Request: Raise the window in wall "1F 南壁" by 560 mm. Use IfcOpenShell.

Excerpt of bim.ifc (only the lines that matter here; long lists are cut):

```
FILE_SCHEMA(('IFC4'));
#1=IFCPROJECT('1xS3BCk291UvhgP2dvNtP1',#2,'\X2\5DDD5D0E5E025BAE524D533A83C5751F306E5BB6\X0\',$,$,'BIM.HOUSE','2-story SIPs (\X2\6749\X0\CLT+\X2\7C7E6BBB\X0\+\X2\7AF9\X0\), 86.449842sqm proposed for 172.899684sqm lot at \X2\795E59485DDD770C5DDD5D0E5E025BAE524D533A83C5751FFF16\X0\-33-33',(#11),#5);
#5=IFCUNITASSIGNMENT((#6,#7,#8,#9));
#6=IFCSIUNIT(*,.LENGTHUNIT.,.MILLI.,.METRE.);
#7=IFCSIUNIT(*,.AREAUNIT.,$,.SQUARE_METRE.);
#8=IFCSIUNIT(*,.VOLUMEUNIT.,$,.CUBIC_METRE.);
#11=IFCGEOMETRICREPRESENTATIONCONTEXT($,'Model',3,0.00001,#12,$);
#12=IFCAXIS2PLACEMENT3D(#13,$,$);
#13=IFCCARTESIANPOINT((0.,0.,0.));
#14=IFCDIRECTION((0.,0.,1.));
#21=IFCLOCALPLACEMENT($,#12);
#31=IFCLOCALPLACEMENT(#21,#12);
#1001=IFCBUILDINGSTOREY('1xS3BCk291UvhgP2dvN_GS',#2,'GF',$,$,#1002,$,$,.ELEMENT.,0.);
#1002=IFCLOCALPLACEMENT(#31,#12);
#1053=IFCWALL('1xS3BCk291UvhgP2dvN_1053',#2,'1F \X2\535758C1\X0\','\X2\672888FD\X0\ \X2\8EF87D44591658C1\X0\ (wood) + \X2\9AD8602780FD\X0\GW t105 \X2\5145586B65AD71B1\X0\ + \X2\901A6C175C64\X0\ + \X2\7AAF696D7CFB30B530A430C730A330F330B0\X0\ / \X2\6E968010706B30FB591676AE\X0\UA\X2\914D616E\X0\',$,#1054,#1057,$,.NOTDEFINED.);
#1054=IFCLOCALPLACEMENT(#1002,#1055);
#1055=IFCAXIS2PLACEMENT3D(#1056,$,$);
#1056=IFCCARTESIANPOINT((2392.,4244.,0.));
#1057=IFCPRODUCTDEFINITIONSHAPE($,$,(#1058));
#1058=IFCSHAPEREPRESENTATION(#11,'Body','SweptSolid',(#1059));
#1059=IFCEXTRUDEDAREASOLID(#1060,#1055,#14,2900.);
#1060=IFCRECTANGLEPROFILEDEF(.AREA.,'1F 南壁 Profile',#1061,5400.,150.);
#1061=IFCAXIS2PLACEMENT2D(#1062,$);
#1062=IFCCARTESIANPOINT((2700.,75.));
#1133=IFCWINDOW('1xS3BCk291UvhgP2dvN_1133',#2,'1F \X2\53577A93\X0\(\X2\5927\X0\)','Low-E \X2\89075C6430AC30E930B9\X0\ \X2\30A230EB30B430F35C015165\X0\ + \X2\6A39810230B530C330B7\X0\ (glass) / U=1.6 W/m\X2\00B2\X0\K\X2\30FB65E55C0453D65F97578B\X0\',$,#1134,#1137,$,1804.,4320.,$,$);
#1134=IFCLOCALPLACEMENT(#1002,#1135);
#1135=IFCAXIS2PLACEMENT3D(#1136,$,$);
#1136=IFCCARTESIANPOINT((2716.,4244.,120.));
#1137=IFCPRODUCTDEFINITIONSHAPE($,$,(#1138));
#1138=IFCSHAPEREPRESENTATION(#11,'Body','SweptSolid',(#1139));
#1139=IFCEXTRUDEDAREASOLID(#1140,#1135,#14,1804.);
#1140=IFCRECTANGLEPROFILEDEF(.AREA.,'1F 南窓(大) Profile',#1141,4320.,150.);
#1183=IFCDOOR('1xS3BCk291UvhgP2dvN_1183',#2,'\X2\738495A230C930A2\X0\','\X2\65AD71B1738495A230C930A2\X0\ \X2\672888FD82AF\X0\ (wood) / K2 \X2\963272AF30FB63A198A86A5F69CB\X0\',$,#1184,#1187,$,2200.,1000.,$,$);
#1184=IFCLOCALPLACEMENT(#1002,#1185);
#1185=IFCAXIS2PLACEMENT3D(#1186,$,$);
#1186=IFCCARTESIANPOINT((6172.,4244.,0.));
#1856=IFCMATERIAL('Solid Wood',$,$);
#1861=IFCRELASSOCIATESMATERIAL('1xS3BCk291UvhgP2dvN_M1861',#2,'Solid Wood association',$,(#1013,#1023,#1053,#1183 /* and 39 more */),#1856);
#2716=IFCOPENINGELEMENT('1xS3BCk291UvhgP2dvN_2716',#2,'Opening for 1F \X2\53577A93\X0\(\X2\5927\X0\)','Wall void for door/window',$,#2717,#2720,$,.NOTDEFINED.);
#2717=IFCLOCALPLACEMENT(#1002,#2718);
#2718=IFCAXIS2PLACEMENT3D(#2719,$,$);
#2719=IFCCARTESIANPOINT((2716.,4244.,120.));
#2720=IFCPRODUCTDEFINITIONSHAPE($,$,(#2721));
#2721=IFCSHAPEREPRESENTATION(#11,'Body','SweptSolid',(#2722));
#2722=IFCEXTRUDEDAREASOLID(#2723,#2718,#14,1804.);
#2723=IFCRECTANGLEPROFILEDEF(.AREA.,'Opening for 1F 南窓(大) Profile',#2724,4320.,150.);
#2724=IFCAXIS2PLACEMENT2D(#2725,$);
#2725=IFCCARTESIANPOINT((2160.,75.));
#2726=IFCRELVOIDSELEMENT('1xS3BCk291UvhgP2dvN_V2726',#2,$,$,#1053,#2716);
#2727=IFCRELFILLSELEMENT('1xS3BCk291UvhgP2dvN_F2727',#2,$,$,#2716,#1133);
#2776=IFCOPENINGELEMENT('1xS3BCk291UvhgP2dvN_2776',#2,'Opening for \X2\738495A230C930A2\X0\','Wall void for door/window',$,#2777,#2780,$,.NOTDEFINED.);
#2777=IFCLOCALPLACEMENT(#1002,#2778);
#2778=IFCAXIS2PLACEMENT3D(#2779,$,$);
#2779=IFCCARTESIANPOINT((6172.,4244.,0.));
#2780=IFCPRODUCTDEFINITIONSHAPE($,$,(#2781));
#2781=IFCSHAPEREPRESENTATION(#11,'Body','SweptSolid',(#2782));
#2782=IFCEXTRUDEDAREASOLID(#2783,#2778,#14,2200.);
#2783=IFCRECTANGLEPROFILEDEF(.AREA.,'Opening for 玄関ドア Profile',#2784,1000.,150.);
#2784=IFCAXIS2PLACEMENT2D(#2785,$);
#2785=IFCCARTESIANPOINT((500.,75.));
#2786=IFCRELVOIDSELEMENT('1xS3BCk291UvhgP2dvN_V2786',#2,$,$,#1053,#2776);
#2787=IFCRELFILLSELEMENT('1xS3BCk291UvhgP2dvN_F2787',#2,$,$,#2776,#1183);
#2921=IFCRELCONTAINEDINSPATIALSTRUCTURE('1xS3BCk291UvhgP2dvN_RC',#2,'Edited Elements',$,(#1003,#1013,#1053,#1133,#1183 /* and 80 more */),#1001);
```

```python
import numpy as np
import ifcopenshell
import ifcopenshell.api.geometry
import ifcopenshell.util.placement
import ifcopenshell.util.unit

model = ifcopenshell.open("bim.ifc")
unit_scale = ifcopenshell.util.unit.calculate_unit_scale(model)

window = model.by_id(1133)
opening = window.FillsVoids[0].RelatingOpeningElement
dz = 560.0

shift = np.array([0.0, 0.0, dz])
# The window is not placed relative to its opening, so move both.
for product in (opening, window):
    matrix = ifcopenshell.util.placement.get_local_placement(product.ObjectPlacement)
    matrix[:3, 3] += shift
    ifcopenshell.api.geometry.edit_object_placement(model, product=product, matrix=matrix, is_si=False)

print(f"moved by {dz * unit_scale:+.3f} m")

model.write("bim_rev.ifc")
```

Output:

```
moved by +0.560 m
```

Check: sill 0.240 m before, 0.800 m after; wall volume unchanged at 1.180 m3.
